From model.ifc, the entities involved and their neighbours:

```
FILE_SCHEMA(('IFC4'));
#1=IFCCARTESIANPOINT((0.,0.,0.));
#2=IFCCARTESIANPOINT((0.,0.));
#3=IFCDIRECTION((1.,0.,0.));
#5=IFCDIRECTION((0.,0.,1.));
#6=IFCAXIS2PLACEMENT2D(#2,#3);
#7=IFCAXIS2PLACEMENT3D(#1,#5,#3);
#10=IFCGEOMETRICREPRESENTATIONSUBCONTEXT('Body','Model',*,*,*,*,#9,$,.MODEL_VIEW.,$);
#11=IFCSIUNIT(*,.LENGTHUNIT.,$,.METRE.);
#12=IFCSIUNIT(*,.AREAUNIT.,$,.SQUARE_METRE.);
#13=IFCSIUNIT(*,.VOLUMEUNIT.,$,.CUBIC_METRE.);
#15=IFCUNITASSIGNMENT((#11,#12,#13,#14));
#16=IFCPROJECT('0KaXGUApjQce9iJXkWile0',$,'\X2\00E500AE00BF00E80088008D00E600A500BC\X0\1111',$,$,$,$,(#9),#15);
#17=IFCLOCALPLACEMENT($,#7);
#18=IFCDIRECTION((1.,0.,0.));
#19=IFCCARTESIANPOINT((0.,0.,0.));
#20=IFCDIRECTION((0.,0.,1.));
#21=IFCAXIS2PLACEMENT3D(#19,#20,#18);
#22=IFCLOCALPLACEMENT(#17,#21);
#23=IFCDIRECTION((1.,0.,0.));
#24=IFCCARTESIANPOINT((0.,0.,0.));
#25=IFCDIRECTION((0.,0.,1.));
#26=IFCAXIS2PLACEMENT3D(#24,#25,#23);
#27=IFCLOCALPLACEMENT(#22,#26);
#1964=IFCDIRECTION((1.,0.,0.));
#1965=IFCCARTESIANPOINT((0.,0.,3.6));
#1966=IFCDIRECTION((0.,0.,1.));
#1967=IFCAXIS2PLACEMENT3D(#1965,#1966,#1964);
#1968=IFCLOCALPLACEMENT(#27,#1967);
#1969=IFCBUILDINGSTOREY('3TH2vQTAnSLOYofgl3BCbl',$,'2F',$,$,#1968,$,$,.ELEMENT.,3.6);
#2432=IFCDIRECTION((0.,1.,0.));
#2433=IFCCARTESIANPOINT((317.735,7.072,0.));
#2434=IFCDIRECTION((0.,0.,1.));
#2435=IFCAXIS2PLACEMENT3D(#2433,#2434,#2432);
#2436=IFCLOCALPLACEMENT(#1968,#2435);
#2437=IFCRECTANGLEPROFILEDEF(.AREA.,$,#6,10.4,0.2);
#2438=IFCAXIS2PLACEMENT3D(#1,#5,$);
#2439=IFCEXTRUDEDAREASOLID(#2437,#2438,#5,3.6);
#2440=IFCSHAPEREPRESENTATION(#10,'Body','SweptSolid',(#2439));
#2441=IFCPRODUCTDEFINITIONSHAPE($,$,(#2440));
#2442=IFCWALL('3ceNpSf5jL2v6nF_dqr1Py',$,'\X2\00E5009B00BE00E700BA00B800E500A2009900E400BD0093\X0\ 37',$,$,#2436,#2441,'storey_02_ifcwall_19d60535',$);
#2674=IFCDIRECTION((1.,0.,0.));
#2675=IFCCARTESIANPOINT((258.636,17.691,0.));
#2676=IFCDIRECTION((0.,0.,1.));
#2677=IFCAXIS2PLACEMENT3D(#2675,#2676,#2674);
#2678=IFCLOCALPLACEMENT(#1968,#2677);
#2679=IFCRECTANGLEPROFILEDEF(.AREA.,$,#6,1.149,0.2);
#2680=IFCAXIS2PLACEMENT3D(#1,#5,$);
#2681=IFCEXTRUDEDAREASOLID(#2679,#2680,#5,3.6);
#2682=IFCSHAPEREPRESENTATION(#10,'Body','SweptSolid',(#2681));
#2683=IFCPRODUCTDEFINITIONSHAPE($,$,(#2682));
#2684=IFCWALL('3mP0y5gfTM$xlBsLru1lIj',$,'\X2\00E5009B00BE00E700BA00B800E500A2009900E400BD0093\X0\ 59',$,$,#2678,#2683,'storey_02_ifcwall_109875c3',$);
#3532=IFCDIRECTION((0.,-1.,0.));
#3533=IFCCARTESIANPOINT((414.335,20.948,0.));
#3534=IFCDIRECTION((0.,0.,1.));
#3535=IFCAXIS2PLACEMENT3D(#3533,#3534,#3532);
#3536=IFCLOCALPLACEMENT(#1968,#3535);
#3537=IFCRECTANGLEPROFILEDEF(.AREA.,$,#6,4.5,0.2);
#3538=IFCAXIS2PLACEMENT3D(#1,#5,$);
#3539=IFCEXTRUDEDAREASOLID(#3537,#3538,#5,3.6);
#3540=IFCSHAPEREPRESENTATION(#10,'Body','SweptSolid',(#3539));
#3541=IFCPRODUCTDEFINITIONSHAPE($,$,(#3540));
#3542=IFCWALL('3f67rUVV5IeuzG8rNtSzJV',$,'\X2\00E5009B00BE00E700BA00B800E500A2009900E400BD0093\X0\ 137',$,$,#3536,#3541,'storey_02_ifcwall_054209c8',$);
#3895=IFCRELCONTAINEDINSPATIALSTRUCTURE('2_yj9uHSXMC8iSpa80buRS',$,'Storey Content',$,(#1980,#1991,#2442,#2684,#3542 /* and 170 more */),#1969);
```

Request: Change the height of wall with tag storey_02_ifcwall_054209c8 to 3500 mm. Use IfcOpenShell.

```python
import ifcopenshell
import ifcopenshell.geom
import ifcopenshell.util.representation
import ifcopenshell.util.shape
import ifcopenshell.util.unit

model = ifcopenshell.open("model.ifc")
unit_scale = ifcopenshell.util.unit.calculate_unit_scale(model)
settings = ifcopenshell.geom.settings()


def volume(element):
    """Net volume in cubic metres, openings subtracted."""
    shape = ifcopenshell.geom.create_shape(settings, element)
    return ifcopenshell.util.shape.get_volume(shape.geometry)


wall = model.by_guid("3f67rUVV5IeuzG8rNtSzJV")
before = volume(wall)

body = ifcopenshell.util.representation.get_representation(wall, "Model", "Body")
solid = body.Items[0]
old_height = solid.Depth
solid.Depth = 3.5 / unit_scale
after = volume(wall)

print(f"height {old_height:g} -> {solid.Depth:g}, volume {before:.3f} -> {after:.3f} m3")

model.write("model_rev.ifc")
```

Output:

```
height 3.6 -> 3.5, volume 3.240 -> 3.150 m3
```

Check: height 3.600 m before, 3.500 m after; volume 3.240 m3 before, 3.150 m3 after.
